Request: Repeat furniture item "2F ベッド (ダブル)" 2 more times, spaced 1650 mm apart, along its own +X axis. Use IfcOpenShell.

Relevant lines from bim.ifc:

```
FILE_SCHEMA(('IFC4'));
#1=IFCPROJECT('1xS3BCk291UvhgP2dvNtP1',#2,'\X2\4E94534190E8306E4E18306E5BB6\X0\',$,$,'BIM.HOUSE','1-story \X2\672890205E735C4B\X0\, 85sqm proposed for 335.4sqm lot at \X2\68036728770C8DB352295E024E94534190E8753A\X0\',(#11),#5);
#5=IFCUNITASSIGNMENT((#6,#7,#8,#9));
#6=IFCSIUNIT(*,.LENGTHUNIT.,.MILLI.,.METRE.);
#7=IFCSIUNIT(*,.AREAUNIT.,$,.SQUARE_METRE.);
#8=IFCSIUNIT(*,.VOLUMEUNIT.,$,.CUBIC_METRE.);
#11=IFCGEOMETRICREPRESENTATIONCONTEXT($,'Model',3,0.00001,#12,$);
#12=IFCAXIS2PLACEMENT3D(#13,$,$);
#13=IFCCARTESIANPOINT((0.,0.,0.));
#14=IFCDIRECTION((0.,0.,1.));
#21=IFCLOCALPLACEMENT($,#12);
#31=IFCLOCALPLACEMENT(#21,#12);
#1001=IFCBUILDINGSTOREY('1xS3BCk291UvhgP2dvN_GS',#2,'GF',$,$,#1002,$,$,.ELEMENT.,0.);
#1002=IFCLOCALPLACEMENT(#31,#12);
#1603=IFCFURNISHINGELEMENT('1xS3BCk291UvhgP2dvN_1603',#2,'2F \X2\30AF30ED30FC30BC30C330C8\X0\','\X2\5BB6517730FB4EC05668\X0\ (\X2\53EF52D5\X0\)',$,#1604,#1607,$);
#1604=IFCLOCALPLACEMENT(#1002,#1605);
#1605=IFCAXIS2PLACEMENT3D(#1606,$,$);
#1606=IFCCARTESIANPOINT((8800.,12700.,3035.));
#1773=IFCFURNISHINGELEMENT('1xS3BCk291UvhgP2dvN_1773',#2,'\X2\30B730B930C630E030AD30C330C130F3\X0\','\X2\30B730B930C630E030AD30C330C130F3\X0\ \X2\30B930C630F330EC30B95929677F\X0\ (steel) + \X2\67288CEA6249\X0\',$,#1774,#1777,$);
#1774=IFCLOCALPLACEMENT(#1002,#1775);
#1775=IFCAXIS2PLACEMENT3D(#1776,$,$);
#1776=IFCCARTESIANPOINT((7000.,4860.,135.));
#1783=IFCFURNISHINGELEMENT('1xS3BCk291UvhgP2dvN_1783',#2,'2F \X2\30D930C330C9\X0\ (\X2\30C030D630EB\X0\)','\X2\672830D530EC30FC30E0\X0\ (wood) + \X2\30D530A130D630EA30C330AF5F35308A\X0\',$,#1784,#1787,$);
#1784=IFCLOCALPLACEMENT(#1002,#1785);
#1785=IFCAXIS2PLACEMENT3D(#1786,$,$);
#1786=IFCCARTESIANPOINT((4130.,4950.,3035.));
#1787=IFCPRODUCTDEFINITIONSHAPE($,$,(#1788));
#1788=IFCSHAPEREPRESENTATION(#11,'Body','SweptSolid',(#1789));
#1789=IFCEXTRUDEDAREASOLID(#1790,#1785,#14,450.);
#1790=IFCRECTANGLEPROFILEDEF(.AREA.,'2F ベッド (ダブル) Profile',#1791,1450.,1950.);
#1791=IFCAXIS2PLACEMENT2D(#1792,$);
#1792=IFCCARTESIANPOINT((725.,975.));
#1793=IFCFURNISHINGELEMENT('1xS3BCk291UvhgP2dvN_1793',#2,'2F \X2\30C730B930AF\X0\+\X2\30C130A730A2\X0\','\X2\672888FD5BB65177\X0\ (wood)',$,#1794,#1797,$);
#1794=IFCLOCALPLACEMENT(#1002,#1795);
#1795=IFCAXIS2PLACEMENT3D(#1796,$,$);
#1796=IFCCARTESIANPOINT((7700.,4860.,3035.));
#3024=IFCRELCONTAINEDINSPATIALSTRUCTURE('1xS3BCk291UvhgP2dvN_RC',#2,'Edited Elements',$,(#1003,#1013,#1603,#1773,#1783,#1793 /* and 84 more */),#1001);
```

```python
import ifcopenshell
import ifcopenshell.api.geometry
import ifcopenshell.api.root
import ifcopenshell.util.element
import ifcopenshell.util.placement
import ifcopenshell.util.unit

model = ifcopenshell.open("bim.ifc")
unit_scale = ifcopenshell.util.unit.calculate_unit_scale(model)


def reuse_history(source, copy):
    """copy_class also copies each property set's owner history, people and application; keep the originals."""
    for rel in copy.IsDefinedBy:
        if rel.is_a("IfcRelDefinesByProperties") and (history := rel.RelatingPropertyDefinition.OwnerHistory):
            rel.RelatingPropertyDefinition.OwnerHistory = source.OwnerHistory
            ifcopenshell.util.element.remove_deep2(model, history)


source = model.by_id(1783)
base = ifcopenshell.util.placement.get_local_placement(source.ObjectPlacement)
step = base[:3, 0] * 1.65 / unit_scale

for i in range(1, 3):
    copy = ifcopenshell.api.root.copy_class(model, product=source)
    copy.Representation = ifcopenshell.util.element.copy_deep(
        model, source.Representation, exclude=["IfcGeometricRepresentationContext", "IfcRepresentationMap"]
    )
    reuse_history(source, copy)
    matrix = base.copy()
    matrix[:3, 3] += i * step
    print("added at", matrix[:3, 3].round(3) + 0.0)
    ifcopenshell.api.geometry.edit_object_placement(model, product=copy, matrix=matrix, is_si=False)

model.write("bim_edited.ifc")
```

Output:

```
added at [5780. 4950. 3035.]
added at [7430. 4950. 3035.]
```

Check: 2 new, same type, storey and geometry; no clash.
